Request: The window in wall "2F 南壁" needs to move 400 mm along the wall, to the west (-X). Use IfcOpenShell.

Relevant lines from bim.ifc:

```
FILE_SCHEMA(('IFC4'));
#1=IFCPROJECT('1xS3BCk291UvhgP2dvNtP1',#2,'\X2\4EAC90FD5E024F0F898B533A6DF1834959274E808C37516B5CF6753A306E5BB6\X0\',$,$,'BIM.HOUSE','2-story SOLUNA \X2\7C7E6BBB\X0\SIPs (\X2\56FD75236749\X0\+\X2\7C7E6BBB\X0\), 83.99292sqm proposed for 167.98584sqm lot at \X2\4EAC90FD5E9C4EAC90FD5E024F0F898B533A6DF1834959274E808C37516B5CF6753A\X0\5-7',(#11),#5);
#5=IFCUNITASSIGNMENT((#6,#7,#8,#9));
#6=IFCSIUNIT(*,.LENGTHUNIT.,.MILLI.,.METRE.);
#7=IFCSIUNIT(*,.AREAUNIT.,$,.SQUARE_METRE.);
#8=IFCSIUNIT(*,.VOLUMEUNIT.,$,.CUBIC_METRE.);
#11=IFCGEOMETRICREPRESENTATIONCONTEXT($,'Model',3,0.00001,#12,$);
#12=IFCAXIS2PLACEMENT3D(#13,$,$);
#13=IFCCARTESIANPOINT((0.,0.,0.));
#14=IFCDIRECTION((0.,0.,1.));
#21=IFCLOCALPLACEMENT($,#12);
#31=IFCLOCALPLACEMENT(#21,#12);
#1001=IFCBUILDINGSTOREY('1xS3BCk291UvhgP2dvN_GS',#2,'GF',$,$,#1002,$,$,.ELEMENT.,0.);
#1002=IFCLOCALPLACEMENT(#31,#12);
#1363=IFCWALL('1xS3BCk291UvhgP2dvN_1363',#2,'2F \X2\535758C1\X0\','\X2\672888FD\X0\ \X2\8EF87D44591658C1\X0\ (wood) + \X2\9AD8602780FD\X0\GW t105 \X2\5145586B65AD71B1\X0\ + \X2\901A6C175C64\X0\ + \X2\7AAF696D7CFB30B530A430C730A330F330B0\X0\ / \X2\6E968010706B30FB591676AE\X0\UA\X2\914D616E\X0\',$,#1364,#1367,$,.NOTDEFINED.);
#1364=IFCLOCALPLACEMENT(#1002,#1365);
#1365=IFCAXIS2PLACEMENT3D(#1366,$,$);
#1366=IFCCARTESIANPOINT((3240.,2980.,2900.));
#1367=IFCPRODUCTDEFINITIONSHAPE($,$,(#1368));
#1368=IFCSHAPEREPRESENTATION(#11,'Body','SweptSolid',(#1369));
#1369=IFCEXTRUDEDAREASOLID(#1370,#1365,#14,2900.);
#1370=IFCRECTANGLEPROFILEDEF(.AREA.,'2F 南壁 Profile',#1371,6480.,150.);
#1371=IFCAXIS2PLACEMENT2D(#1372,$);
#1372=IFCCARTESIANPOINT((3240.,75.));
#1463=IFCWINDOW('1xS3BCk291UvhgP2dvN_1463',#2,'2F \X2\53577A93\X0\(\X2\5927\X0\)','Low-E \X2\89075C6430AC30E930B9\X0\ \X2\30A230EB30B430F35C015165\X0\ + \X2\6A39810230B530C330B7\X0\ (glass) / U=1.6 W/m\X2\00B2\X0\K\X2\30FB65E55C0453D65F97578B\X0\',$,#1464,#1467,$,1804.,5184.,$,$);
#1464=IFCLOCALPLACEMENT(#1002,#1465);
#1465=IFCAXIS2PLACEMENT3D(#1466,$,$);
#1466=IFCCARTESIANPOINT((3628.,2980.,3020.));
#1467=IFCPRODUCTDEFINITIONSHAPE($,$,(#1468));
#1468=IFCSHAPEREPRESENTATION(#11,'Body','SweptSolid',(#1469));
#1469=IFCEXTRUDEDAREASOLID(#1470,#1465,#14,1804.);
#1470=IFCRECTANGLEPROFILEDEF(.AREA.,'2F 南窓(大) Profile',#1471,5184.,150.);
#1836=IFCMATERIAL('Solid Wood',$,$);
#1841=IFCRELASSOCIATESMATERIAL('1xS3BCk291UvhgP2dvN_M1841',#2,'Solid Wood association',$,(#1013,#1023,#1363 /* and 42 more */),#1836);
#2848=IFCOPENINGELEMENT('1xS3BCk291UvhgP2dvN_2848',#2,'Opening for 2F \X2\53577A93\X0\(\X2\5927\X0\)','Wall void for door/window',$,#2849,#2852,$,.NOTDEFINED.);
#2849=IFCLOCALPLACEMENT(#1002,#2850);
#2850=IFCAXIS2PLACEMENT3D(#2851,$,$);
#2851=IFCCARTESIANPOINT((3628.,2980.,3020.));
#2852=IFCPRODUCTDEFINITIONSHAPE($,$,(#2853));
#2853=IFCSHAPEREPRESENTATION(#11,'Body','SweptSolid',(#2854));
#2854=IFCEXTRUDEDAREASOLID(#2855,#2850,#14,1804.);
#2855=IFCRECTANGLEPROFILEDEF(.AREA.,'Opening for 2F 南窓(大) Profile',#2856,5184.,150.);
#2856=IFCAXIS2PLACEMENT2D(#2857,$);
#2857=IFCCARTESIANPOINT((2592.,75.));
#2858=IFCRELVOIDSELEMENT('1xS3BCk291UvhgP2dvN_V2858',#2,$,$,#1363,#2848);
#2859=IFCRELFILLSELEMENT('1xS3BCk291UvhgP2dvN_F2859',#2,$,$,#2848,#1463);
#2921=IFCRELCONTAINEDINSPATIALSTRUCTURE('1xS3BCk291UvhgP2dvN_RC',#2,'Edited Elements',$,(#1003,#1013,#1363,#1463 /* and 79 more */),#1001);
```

```python
import ifcopenshell
import ifcopenshell.api.geometry
import ifcopenshell.util.placement
import ifcopenshell.util.unit

model = ifcopenshell.open("bim.ifc")
unit_scale = ifcopenshell.util.unit.calculate_unit_scale(model)

window = model.by_guid("1xS3BCk291UvhgP2dvN_1463")
opening = window.FillsVoids[0].RelatingOpeningElement
wall = opening.VoidsElements[0].RelatingBuildingElement

wall_matrix = ifcopenshell.util.placement.get_local_placement(wall.ObjectPlacement)
shift = wall_matrix[:3, 0] * -0.4 / unit_scale
before = ifcopenshell.util.placement.get_local_placement(window.ObjectPlacement)[:3, 3].copy()

# The window is not placed relative to its opening, so move both.
for product in (opening, window):
    matrix = ifcopenshell.util.placement.get_local_placement(product.ObjectPlacement)
    matrix[:3, 3] += shift
    ifcopenshell.api.geometry.edit_object_placement(model, product=product, matrix=matrix, is_si=False)

after = ifcopenshell.util.placement.get_local_placement(window.ObjectPlacement)[:3, 3]
print("window moved by", (after - before).round(3) + 0.0)

model.write("bim_edited.ifc")
```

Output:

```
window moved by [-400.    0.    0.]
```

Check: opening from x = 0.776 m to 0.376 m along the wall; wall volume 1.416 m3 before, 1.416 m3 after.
